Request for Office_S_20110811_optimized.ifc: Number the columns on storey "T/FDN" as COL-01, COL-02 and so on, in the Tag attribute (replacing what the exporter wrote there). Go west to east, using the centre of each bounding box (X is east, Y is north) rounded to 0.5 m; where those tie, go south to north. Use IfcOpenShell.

First a look at what the model holds.

```python
import ifcopenshell
import ifcopenshell.util.element
import ifcopenshell.util.placement

model = ifcopenshell.open("Office_S_20110811_optimized.ifc")
print(model.schema)
storey = next(s for s in model.by_type("IfcBuildingStorey") if s.Name == "T/FDN")
columns = [e for e in ifcopenshell.util.element.get_decomposition(storey) if e.is_a("IfcColumn")]
for e in sorted(columns, key=lambda e: e.id()):
    origin = ifcopenshell.util.placement.get_local_placement(e.ObjectPlacement)[:3, 3]
    print(e.id(), e.Tag, e.Name, origin.round(2) + 0.0, sep=" | ")
```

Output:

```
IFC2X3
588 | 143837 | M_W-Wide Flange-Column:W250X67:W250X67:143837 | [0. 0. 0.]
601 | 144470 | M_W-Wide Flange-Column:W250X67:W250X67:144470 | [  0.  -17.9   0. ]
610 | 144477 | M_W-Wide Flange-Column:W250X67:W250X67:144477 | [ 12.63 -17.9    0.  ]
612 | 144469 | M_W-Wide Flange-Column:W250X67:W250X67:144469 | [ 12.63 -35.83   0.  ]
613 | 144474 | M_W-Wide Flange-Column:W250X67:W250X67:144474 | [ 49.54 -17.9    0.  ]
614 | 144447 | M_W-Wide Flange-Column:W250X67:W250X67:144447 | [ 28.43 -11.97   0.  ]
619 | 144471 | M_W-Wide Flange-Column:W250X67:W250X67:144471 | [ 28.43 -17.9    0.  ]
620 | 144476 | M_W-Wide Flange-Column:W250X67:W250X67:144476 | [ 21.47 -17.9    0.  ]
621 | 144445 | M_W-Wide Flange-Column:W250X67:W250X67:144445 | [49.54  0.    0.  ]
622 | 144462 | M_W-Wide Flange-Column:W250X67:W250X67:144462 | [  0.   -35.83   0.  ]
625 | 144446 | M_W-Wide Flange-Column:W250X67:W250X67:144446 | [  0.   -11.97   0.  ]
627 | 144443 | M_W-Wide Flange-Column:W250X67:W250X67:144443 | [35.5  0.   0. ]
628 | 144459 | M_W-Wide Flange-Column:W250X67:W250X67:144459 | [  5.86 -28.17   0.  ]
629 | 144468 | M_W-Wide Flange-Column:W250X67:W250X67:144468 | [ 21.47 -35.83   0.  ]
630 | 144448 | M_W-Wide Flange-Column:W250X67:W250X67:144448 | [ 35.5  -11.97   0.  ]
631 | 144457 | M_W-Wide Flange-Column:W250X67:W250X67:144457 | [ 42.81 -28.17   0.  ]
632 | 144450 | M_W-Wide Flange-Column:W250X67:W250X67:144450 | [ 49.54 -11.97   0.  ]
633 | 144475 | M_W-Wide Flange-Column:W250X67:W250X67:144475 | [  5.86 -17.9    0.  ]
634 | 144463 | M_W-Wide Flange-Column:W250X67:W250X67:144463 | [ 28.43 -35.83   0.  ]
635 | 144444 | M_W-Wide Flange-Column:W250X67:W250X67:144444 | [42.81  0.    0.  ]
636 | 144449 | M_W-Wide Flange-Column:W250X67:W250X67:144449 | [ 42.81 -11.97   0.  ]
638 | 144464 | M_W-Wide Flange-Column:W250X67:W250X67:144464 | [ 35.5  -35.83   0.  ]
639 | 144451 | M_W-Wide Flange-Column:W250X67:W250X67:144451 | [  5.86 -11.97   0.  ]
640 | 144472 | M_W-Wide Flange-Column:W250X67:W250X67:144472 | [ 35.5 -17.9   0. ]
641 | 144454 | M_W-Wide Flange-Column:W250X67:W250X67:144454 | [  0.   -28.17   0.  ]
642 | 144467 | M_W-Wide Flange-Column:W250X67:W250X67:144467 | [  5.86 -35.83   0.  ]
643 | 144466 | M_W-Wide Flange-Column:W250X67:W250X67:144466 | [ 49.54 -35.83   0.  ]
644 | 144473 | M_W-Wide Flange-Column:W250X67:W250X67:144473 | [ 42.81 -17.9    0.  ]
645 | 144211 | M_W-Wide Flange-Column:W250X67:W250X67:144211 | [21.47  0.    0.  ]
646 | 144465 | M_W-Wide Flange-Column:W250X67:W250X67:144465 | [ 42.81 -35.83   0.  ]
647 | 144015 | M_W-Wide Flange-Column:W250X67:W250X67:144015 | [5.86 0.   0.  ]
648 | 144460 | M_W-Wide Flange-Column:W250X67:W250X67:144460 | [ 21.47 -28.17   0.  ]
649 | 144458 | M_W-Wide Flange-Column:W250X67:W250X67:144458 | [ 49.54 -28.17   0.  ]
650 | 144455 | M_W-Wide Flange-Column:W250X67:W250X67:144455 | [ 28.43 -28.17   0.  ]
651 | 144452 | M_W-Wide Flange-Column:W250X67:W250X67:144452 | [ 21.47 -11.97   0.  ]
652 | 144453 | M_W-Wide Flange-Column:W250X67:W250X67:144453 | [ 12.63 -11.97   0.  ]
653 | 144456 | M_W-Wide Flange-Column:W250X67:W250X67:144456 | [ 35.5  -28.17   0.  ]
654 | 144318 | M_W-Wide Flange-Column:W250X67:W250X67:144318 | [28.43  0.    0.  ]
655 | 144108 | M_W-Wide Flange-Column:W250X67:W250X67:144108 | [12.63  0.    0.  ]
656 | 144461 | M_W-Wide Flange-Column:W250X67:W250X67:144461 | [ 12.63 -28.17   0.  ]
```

```python
import ifcopenshell
import ifcopenshell.geom
import ifcopenshell.util.element
import ifcopenshell.util.shape

model = ifcopenshell.open("Office_S_20110811_optimized.ifc")
settings = ifcopenshell.geom.settings()
settings.set("use-world-coords", True)


def centre(element):
    shape = ifcopenshell.geom.create_shape(settings, element)
    return ifcopenshell.util.shape.get_bbox_centroid(shape.geometry)


storey = next(s for s in model.by_type("IfcBuildingStorey") if s.Name == "T/FDN")
columns = [e for e in ifcopenshell.util.element.get_decomposition(storey) if e.is_a("IfcColumn")]

# Insertion points can sit at a corner or the storey origin, so sort by the geometry (in metres).
centres = {e: centre(e) for e in columns}
columns.sort(key=lambda e: (round(centres[e][0] / 0.5), centres[e][1]))

for i, e in enumerate(columns, start=1):
    number = f"COL-{i:02d}"
    e.Tag = number
    print(e.id(), number)

model.write("Office_S_20110811_optimized_v2.ifc")
```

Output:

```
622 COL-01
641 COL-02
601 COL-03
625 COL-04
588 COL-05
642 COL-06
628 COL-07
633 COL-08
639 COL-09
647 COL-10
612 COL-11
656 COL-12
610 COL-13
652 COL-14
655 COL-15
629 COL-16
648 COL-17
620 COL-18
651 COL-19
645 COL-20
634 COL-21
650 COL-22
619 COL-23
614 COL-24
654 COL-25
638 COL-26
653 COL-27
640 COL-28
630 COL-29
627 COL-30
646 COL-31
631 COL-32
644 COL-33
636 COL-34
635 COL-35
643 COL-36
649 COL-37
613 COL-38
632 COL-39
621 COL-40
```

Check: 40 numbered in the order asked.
